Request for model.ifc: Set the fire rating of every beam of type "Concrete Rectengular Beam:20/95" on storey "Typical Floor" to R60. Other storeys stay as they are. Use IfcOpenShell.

First a look at what the model holds.

```python
import ifcopenshell
import ifcopenshell.util.element

model = ifcopenshell.open("model.ifc")
print(model.schema)
storey = next(s for s in model.by_type("IfcBuildingStorey") if s.Name == "Typical Floor")
beams = [e for e in ifcopenshell.util.element.get_decomposition(storey) if e.is_a("IfcBeam")]
seen = {}
for e in beams:
    element_type = ifcopenshell.util.element.get_type(e)
    key = (element_type.Name if element_type != e and element_type else None, ifcopenshell.util.element.get_pset(e, "Pset_BeamCommon", "FireRating"))
    seen[key] = seen.get(key, 0) + 1
for (name, value), count in sorted(seen.items(), key=str):
    print(count, "x", name, "|", value)
```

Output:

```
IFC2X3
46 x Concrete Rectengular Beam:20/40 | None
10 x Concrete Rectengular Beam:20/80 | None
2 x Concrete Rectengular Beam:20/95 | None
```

```python
import ifcopenshell
import ifcopenshell.api.pset
import ifcopenshell.util.element

model = ifcopenshell.open("model.ifc")

storey = next(s for s in model.by_type("IfcBuildingStorey") if s.Name == "Typical Floor")
beams = [e for e in ifcopenshell.util.element.get_decomposition(storey) if e.is_a("IfcBeam")]

count = 0
for e in beams:
    element_type = ifcopenshell.util.element.get_type(e)
    if element_type in (None, e) or element_type.Name != "Concrete Rectengular Beam:20/95":
        continue
    # add_pset returns the element's existing set when there is one.
    pset = ifcopenshell.api.pset.add_pset(model, product=e, name="Pset_BeamCommon")
    ifcopenshell.api.pset.edit_pset(model, pset=pset, properties={"FireRating": "R60"})
    count += 1

print(count, "beams updated")

model.write("model_edited.ifc")
```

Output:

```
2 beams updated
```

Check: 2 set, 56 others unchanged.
